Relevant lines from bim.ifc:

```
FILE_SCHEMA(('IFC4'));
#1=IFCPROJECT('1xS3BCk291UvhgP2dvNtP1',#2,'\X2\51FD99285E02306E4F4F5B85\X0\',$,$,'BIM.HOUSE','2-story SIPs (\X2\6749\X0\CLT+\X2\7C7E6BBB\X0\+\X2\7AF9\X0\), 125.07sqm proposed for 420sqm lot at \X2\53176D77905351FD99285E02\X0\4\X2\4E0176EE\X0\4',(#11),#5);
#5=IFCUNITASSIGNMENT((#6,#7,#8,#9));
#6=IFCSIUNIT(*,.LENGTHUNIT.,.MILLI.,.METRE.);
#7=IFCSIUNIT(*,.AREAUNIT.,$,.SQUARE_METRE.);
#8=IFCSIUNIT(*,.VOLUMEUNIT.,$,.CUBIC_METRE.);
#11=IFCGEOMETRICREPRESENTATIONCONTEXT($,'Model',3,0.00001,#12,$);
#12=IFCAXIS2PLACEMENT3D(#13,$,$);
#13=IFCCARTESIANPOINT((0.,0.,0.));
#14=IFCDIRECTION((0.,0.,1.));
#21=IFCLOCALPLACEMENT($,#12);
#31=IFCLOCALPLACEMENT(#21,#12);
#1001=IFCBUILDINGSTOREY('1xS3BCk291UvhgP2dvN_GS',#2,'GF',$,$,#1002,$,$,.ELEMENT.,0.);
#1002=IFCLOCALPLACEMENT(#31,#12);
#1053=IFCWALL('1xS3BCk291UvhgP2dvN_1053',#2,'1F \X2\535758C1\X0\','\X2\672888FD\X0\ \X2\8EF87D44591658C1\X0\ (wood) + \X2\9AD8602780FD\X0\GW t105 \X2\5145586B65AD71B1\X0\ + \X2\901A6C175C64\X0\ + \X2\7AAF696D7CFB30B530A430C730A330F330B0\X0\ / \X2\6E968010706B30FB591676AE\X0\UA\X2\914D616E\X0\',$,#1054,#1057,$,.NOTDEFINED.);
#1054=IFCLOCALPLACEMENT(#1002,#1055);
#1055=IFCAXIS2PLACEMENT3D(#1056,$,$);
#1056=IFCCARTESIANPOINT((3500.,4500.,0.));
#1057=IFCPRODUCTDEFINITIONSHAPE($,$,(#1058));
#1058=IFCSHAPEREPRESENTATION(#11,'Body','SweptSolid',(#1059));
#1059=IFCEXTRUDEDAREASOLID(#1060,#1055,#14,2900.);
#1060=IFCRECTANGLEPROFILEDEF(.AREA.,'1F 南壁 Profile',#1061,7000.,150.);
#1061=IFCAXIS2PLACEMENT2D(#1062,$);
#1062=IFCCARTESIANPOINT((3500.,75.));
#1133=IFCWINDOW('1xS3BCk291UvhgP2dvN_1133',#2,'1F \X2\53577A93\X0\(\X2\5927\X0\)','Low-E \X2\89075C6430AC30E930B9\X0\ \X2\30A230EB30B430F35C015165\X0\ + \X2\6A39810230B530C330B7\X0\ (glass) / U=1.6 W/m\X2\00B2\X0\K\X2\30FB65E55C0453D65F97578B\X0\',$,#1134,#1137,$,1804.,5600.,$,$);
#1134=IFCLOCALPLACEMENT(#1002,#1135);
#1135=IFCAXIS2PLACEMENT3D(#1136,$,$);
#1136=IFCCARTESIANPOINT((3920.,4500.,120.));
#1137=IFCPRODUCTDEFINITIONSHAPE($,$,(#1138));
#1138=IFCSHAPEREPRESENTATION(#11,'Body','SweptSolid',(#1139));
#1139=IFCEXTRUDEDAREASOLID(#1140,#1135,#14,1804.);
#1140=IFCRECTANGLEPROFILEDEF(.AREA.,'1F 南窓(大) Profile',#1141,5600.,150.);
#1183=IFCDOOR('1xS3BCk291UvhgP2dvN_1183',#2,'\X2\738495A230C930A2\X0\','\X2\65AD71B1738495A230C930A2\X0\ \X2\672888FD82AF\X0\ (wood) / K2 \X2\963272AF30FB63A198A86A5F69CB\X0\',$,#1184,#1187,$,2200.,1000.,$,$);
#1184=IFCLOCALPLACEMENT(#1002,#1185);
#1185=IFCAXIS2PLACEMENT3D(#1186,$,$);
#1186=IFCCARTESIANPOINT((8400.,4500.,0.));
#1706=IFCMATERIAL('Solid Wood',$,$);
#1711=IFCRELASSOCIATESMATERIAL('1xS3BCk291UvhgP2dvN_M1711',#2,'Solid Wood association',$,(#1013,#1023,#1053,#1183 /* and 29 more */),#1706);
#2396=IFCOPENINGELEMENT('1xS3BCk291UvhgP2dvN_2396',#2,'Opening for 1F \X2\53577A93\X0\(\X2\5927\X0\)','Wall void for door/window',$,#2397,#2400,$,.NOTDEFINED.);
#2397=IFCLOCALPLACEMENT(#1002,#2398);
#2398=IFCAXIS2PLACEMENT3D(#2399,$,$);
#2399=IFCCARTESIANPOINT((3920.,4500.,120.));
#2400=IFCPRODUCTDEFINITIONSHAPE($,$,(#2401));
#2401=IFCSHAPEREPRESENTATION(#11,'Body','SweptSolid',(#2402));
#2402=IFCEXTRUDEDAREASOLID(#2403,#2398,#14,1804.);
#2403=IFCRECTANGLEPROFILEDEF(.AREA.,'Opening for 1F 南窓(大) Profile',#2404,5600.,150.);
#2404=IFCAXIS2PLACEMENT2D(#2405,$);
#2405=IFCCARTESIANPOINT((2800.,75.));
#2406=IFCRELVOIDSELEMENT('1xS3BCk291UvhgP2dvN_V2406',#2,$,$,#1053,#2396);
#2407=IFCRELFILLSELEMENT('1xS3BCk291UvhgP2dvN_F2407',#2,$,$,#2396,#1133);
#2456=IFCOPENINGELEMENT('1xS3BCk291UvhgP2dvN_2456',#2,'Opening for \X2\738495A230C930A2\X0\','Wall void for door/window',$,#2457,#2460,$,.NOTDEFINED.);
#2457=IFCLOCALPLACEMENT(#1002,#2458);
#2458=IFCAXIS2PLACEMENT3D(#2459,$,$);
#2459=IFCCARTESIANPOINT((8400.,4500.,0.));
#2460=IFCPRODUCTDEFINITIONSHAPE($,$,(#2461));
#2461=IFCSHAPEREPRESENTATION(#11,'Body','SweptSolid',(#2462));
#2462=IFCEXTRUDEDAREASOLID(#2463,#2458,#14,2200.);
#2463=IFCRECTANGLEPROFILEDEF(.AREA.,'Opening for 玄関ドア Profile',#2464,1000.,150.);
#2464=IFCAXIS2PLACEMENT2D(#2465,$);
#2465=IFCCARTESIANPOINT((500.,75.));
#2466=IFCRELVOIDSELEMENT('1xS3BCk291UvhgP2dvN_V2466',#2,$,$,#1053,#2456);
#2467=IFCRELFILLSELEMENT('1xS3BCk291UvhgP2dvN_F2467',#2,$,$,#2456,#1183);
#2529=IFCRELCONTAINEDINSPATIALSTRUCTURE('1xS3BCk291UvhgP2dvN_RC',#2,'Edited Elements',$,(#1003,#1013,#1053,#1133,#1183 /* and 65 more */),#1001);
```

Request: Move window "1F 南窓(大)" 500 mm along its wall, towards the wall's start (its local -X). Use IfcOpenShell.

```python
import ifcopenshell
import ifcopenshell.api.geometry
import ifcopenshell.util.placement

model = ifcopenshell.open("bim.ifc")

window = model.by_guid("1xS3BCk291UvhgP2dvN_1133")
opening = window.FillsVoids[0].RelatingOpeningElement
wall = opening.VoidsElements[0].RelatingBuildingElement

wall_matrix = ifcopenshell.util.placement.get_local_placement(wall.ObjectPlacement)
shift = wall_matrix[:3, 0] * -500.0
before = ifcopenshell.util.placement.get_local_placement(window.ObjectPlacement)[:3, 3].copy()

# The window is not placed relative to its opening, so move both.
for product in (opening, window):
    matrix = ifcopenshell.util.placement.get_local_placement(product.ObjectPlacement)
    matrix[:3, 3] += shift
    ifcopenshell.api.geometry.edit_object_placement(model, product=product, matrix=matrix, is_si=False)

after = ifcopenshell.util.placement.get_local_placement(window.ObjectPlacement)[:3, 3]
print("window moved by", (after - before).round(3) + 0.0)

model.write("bim_v2.ifc")
```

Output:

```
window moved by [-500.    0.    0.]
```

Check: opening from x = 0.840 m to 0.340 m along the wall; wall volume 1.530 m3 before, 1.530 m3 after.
